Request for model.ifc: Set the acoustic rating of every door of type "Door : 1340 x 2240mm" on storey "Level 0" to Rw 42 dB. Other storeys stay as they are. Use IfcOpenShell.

First a look at what the model holds.

```python
import ifcopenshell
import ifcopenshell.util.element

model = ifcopenshell.open("model.ifc")
print(model.schema)
storey = next(s for s in model.by_type("IfcBuildingStorey") if s.Name == "Level 0")
doors = [e for e in ifcopenshell.util.element.get_decomposition(storey) if e.is_a("IfcDoor")]
seen = {}
for e in doors:
    element_type = ifcopenshell.util.element.get_type(e)
    key = (element_type.Name if element_type != e and element_type else None, ifcopenshell.util.element.get_pset(e, "Pset_DoorCommon", "AcousticRating"))
    seen[key] = seen.get(key, 0) + 1
for (name, value), count in sorted(seen.items(), key=str):
    print(count, "x", name, "|", value)
```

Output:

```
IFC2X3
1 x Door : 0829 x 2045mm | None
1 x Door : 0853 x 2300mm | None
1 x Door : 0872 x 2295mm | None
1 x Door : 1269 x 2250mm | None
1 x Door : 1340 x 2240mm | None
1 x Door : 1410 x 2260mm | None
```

```python
import ifcopenshell
import ifcopenshell.api.pset
import ifcopenshell.util.element

model = ifcopenshell.open("model.ifc")

storey = next(s for s in model.by_type("IfcBuildingStorey") if s.Name == "Level 0")
doors = [e for e in ifcopenshell.util.element.get_decomposition(storey) if e.is_a("IfcDoor")]

count = 0
for e in doors:
    element_type = ifcopenshell.util.element.get_type(e)
    if element_type in (None, e) or element_type.Name != "Door : 1340 x 2240mm":
        continue
    # add_pset returns the element's existing set when there is one.
    pset = ifcopenshell.api.pset.add_pset(model, product=e, name="Pset_DoorCommon")
    ifcopenshell.api.pset.edit_pset(model, pset=pset, properties={"AcousticRating": "Rw 42 dB"})
    count += 1

print(count, "doors updated")

model.write("model-out.ifc")
```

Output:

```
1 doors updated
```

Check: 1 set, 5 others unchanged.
